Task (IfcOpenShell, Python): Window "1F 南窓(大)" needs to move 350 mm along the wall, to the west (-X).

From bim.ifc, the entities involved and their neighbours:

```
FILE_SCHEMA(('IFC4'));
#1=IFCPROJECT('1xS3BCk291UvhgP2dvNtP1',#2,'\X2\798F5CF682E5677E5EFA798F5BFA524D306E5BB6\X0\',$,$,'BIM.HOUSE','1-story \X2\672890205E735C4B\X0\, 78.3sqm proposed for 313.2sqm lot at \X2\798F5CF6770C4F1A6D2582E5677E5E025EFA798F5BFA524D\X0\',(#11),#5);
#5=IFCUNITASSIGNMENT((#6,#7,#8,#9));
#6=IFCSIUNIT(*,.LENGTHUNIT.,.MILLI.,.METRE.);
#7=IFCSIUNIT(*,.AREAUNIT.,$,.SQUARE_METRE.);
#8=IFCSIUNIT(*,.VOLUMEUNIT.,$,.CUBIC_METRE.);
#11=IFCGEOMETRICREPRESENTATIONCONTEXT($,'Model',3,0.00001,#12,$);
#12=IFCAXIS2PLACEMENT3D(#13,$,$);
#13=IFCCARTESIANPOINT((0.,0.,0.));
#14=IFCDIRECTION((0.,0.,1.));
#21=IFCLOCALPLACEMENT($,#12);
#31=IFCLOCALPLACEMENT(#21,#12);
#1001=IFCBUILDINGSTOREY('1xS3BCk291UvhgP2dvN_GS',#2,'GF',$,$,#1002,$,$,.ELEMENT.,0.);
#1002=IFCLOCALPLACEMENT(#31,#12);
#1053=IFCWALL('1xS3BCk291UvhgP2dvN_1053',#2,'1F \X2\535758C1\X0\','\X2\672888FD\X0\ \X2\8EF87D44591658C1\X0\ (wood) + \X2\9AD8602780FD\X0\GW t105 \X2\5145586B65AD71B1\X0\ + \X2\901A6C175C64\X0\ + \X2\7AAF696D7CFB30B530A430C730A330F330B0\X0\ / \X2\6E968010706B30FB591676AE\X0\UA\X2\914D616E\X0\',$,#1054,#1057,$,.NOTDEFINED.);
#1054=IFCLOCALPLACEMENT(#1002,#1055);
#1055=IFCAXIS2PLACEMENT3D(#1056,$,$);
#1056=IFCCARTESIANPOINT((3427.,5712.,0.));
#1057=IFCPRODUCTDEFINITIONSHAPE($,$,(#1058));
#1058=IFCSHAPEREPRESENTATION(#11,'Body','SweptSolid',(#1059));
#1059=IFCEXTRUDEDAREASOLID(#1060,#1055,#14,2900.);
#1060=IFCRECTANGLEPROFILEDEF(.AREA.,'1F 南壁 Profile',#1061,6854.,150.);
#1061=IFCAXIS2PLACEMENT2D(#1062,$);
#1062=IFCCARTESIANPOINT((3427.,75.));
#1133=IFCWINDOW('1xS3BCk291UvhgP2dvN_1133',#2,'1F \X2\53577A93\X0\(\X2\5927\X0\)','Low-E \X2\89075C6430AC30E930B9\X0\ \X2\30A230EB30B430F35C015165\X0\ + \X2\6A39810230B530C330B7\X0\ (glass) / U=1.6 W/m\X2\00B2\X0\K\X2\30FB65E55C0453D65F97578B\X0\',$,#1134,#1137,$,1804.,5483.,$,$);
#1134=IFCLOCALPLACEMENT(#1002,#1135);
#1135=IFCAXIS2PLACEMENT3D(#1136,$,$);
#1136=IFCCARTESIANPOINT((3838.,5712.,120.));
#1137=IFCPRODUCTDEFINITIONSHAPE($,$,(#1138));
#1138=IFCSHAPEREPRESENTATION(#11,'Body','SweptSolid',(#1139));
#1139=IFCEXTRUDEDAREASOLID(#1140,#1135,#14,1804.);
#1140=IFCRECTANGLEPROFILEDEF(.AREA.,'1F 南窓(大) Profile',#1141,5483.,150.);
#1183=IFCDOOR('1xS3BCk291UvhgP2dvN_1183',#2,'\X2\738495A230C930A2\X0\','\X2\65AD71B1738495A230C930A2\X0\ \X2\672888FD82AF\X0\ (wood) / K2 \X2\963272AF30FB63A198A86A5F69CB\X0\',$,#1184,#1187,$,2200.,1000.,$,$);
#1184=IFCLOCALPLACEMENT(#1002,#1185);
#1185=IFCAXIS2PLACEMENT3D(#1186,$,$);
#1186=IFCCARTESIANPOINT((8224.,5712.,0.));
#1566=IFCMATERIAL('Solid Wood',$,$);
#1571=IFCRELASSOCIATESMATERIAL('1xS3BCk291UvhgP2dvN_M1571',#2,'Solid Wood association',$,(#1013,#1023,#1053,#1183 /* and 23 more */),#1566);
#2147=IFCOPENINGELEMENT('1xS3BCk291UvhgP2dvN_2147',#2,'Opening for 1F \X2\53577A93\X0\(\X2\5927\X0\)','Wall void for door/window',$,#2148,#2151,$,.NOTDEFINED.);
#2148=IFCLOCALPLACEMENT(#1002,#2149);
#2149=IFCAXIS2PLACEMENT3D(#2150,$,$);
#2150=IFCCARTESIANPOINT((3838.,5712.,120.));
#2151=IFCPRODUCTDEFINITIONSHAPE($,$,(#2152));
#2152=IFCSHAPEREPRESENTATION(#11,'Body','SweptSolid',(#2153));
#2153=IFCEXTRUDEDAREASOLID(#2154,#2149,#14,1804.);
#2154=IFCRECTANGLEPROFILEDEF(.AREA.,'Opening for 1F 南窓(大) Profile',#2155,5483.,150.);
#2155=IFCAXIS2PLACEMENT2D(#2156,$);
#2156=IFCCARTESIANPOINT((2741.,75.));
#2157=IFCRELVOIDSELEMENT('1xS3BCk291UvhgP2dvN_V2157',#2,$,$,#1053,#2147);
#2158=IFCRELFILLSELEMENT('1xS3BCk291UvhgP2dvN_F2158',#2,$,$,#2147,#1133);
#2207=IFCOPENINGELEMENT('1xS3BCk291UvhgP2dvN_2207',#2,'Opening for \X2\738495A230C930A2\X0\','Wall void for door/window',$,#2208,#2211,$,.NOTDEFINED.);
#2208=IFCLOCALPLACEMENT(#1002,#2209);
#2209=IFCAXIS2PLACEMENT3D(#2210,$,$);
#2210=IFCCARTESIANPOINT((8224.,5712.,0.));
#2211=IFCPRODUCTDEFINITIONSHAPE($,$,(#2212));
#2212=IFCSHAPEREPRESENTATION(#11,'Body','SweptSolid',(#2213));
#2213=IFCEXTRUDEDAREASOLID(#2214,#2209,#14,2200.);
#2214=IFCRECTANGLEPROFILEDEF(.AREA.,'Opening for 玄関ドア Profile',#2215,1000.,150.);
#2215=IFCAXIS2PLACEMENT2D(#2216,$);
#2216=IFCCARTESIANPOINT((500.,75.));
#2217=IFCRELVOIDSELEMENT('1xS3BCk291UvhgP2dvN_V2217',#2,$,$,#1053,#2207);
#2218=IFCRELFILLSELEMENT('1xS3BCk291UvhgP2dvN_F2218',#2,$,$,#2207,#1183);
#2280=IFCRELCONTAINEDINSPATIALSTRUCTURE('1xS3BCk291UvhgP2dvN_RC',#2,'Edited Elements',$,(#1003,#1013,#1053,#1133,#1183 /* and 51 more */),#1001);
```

```python
import ifcopenshell
import ifcopenshell.api.geometry
import ifcopenshell.util.placement
import ifcopenshell.util.unit

model = ifcopenshell.open("bim.ifc")
unit_scale = ifcopenshell.util.unit.calculate_unit_scale(model)

window = model.by_guid("1xS3BCk291UvhgP2dvN_1133")
opening = window.FillsVoids[0].RelatingOpeningElement
wall = opening.VoidsElements[0].RelatingBuildingElement

wall_matrix = ifcopenshell.util.placement.get_local_placement(wall.ObjectPlacement)
shift = wall_matrix[:3, 0] * -0.35 / unit_scale
before = ifcopenshell.util.placement.get_local_placement(window.ObjectPlacement)[:3, 3].copy()

# The window is not placed relative to its opening, so move both.
for product in (opening, window):
    matrix = ifcopenshell.util.placement.get_local_placement(product.ObjectPlacement)
    matrix[:3, 3] += shift
    ifcopenshell.api.geometry.edit_object_placement(model, product=product, matrix=matrix, is_si=False)

after = ifcopenshell.util.placement.get_local_placement(window.ObjectPlacement)[:3, 3]
print("window moved by", (after - before).round(3) + 0.0)

model.write("bim_rev.ifc")
```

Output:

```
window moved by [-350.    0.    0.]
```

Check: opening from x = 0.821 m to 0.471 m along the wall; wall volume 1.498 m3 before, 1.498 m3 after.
